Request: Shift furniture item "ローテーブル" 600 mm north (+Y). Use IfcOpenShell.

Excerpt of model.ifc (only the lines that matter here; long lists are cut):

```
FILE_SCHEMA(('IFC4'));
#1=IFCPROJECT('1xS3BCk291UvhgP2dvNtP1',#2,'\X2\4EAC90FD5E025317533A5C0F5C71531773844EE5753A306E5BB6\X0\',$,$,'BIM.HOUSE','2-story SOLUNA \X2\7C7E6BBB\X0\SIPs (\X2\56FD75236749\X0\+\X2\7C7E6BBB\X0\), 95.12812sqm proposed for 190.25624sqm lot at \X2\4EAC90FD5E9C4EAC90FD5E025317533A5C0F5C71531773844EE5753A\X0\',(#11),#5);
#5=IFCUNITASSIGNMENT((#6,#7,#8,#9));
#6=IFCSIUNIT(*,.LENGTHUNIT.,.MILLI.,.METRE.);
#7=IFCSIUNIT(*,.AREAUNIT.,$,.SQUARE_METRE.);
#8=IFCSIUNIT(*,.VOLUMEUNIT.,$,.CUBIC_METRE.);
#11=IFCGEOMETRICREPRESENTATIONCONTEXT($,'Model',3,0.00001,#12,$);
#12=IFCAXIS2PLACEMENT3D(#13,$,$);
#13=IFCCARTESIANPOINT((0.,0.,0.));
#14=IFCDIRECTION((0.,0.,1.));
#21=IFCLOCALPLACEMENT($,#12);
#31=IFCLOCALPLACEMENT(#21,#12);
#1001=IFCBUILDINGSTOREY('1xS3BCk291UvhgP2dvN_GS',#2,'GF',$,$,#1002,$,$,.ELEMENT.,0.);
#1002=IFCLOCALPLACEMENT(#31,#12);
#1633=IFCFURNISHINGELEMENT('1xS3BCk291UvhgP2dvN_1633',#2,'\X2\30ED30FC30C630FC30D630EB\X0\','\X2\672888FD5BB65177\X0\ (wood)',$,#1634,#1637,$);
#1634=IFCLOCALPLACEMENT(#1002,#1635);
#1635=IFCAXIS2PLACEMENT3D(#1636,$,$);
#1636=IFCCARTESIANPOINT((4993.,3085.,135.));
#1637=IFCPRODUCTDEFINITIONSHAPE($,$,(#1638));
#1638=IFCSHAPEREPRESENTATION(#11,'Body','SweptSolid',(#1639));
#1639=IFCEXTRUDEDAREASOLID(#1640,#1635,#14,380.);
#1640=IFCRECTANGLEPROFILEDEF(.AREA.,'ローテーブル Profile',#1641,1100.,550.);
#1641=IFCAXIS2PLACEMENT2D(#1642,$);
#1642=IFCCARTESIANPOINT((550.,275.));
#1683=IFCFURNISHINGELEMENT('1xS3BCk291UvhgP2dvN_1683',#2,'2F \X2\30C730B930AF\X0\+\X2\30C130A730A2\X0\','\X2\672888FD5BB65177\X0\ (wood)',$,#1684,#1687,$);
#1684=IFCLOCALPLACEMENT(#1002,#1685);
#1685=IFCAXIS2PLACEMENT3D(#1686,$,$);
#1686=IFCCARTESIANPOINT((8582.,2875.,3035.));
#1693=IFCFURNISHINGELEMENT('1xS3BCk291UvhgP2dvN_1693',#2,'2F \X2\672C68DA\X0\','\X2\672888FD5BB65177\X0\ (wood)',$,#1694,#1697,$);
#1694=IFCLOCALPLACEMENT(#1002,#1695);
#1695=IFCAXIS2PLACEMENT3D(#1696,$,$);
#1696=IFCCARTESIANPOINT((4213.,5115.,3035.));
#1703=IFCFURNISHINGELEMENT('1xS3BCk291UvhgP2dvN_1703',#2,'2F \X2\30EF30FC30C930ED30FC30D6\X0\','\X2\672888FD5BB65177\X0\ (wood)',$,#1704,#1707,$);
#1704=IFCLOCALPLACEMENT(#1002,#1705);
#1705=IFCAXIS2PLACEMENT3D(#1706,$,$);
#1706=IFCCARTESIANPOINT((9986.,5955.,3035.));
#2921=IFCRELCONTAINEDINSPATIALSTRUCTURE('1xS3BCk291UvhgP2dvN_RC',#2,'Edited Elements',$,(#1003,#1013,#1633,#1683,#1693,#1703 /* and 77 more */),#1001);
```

```python
import ifcopenshell
import ifcopenshell.api.geometry
import ifcopenshell.util.placement
import ifcopenshell.util.unit

model = ifcopenshell.open("model.ifc")
unit_scale = ifcopenshell.util.unit.calculate_unit_scale(model)

item = model.by_id(1633)
matrix = ifcopenshell.util.placement.get_local_placement(item.ObjectPlacement)
matrix[1, 3] += 0.6 / unit_scale
ifcopenshell.api.geometry.edit_object_placement(model, product=item, matrix=matrix, is_si=False)

print(ifcopenshell.util.placement.get_local_placement(item.ObjectPlacement).round(3) + 0.0)

model.write("model_updated.ifc")
```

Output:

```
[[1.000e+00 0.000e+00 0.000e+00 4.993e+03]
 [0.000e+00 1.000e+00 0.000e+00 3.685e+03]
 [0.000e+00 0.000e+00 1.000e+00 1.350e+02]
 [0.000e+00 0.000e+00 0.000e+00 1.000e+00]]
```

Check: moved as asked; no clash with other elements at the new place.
